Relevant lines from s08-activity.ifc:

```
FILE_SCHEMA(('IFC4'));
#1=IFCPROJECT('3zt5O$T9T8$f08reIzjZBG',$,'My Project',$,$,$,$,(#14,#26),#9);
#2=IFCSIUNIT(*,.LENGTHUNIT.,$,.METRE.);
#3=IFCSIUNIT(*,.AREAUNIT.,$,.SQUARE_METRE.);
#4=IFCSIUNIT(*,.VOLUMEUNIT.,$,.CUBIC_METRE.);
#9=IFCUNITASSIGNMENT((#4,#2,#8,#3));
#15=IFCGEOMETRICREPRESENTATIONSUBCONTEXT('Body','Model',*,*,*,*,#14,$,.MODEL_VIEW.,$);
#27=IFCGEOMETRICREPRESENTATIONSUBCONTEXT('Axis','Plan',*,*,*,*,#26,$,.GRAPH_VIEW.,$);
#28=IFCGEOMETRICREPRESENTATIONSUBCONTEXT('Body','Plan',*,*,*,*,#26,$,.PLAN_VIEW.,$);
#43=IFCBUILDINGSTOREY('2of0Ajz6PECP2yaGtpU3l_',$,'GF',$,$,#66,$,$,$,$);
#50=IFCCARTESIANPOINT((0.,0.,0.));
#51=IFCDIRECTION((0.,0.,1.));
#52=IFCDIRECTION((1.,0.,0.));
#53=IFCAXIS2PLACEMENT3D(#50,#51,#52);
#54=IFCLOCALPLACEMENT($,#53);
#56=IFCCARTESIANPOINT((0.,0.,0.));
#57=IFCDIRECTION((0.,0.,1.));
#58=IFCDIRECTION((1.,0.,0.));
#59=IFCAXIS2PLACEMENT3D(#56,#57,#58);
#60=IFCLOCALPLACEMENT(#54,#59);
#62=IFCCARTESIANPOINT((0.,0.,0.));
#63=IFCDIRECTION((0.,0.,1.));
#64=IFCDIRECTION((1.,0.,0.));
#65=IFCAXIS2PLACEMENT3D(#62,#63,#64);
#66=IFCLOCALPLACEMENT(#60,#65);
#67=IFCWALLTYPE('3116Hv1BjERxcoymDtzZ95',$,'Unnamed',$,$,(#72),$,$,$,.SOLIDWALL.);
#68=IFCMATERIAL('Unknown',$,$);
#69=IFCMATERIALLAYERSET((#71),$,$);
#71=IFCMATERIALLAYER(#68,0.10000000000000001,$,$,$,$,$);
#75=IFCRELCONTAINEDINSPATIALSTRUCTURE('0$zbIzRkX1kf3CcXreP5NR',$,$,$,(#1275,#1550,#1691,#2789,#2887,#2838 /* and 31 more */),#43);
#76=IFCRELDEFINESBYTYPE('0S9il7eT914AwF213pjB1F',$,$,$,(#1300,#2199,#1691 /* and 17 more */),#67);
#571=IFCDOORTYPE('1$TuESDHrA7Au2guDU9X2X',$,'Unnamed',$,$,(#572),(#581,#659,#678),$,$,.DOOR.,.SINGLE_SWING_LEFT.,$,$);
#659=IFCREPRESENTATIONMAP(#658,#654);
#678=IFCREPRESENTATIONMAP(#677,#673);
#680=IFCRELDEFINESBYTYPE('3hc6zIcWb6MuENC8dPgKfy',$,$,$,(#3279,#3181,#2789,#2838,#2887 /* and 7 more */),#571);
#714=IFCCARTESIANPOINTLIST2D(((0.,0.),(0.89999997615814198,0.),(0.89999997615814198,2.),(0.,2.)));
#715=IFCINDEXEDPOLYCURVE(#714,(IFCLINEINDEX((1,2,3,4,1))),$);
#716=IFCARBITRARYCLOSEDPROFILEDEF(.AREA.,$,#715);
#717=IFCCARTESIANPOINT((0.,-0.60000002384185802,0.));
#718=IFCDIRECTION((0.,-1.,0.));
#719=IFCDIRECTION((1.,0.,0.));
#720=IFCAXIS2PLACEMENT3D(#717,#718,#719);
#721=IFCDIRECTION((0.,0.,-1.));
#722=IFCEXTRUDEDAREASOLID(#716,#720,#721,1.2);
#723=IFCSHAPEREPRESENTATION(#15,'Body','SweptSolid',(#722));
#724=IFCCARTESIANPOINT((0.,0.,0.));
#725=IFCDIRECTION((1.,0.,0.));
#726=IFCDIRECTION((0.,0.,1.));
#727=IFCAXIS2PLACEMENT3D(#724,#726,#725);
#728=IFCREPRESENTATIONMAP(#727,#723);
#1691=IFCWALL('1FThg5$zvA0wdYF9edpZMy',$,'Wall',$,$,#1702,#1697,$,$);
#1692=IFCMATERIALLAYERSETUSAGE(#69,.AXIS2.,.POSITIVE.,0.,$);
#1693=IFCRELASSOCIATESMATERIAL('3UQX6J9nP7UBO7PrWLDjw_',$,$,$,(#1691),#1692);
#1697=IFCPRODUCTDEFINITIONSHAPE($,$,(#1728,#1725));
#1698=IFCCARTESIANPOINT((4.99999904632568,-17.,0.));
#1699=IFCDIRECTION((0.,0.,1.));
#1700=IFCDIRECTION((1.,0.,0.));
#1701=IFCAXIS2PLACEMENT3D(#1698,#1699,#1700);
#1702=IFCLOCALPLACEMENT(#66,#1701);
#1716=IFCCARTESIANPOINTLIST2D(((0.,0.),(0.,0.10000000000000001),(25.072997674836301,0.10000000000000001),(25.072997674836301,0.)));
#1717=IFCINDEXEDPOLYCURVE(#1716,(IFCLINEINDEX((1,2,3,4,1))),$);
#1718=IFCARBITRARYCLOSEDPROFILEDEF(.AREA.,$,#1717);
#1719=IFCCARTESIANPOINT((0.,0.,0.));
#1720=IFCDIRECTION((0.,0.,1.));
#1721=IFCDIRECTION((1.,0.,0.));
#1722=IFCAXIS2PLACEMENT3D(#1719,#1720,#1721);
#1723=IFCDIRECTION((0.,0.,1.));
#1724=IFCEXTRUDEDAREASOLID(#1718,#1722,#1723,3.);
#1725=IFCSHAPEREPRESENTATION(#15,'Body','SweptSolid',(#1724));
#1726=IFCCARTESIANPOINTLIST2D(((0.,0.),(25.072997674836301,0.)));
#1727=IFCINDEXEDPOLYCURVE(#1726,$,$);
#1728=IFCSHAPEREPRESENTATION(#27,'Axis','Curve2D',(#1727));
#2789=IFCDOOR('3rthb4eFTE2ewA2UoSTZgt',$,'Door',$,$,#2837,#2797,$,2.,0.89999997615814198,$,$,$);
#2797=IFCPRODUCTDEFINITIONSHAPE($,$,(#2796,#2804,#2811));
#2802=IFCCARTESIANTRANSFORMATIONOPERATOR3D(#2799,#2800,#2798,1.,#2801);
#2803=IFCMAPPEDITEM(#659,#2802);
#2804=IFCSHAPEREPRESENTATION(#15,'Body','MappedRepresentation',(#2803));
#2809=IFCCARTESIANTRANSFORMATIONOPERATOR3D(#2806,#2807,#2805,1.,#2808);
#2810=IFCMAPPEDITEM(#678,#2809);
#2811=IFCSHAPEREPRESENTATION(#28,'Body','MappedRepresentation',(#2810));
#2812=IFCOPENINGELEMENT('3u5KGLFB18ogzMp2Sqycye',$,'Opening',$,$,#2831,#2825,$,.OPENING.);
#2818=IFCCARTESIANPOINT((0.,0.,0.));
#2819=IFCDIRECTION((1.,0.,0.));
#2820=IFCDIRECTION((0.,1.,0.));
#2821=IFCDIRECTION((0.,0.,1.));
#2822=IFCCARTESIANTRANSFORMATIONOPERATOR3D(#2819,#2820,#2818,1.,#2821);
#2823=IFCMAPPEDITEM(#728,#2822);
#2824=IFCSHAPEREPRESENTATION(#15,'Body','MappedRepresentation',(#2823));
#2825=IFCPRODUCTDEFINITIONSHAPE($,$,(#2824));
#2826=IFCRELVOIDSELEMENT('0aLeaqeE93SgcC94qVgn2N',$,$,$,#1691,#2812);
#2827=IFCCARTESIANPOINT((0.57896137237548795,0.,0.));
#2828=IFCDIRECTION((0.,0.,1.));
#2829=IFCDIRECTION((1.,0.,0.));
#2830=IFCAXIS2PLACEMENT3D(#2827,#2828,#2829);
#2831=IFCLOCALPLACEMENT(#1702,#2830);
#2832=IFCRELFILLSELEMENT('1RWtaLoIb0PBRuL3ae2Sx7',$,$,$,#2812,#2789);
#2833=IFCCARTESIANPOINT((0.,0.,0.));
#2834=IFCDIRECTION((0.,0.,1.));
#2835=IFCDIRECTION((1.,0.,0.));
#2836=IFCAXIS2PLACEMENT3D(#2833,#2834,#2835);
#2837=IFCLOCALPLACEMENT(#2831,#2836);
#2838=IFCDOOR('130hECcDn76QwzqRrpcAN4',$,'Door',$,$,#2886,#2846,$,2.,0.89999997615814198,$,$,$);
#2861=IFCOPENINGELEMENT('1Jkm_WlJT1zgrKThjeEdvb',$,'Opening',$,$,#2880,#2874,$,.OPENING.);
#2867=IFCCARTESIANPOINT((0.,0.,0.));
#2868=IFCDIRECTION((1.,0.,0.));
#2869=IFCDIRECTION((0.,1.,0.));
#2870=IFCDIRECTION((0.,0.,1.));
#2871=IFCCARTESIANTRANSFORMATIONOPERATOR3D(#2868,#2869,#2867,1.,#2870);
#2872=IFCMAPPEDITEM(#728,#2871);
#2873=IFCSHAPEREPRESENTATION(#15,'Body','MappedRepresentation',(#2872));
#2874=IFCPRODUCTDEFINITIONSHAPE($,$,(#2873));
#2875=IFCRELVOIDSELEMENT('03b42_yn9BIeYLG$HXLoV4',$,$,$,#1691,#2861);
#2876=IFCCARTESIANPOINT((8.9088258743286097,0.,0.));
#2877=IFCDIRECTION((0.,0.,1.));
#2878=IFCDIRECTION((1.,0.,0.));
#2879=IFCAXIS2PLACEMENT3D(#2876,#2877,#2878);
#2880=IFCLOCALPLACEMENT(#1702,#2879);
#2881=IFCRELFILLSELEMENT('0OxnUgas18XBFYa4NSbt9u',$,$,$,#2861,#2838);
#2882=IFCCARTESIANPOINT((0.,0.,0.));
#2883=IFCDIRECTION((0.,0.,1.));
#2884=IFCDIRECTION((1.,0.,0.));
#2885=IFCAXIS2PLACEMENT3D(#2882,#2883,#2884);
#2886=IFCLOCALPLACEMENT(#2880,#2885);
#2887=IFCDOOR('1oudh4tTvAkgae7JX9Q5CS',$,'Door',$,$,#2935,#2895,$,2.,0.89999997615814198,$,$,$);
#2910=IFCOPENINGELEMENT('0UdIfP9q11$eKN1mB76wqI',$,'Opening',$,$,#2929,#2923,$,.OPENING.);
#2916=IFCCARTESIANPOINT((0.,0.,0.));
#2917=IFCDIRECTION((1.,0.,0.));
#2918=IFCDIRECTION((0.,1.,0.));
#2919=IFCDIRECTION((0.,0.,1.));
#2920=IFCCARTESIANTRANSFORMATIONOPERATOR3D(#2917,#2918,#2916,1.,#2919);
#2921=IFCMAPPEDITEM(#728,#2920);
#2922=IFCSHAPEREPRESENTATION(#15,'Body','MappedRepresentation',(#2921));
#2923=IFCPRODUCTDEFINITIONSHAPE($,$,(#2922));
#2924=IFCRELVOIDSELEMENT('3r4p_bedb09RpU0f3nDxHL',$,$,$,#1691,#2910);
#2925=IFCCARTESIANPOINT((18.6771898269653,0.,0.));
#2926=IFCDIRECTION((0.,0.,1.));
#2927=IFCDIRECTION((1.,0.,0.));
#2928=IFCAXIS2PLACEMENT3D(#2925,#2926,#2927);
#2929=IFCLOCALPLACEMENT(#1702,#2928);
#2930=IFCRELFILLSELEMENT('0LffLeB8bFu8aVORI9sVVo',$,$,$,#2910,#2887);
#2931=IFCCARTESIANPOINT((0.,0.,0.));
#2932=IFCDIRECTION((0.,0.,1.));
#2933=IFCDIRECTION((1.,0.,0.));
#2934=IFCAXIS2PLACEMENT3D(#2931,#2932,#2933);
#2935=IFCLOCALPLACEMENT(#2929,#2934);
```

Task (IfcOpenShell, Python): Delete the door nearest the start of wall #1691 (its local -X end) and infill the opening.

```python
import ifcopenshell
import ifcopenshell.api.feature
import ifcopenshell.api.root
import ifcopenshell.geom
import ifcopenshell.util.shape

model = ifcopenshell.open("s08-activity.ifc")
settings = ifcopenshell.geom.settings()


def volume(element):
    """Net volume in cubic metres, openings subtracted."""
    shape = ifcopenshell.geom.create_shape(settings, element)
    return ifcopenshell.util.shape.get_volume(shape.geometry)


door = model.by_guid("3rthb4eFTE2ewA2UoSTZgt")
opening = door.FillsVoids[0].RelatingOpeningElement
wall = opening.VoidsElements[0].RelatingBuildingElement
before = volume(wall)

ifcopenshell.api.root.remove_product(model, product=door)
ifcopenshell.api.feature.remove_feature(model, feature=opening)

after = volume(wall)

print(f"wall volume {before:.3f} -> {after:.3f} m3")

model.write("s08-activity_rev.ifc")
```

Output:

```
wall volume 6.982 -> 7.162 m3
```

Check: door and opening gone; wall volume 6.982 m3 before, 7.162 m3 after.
